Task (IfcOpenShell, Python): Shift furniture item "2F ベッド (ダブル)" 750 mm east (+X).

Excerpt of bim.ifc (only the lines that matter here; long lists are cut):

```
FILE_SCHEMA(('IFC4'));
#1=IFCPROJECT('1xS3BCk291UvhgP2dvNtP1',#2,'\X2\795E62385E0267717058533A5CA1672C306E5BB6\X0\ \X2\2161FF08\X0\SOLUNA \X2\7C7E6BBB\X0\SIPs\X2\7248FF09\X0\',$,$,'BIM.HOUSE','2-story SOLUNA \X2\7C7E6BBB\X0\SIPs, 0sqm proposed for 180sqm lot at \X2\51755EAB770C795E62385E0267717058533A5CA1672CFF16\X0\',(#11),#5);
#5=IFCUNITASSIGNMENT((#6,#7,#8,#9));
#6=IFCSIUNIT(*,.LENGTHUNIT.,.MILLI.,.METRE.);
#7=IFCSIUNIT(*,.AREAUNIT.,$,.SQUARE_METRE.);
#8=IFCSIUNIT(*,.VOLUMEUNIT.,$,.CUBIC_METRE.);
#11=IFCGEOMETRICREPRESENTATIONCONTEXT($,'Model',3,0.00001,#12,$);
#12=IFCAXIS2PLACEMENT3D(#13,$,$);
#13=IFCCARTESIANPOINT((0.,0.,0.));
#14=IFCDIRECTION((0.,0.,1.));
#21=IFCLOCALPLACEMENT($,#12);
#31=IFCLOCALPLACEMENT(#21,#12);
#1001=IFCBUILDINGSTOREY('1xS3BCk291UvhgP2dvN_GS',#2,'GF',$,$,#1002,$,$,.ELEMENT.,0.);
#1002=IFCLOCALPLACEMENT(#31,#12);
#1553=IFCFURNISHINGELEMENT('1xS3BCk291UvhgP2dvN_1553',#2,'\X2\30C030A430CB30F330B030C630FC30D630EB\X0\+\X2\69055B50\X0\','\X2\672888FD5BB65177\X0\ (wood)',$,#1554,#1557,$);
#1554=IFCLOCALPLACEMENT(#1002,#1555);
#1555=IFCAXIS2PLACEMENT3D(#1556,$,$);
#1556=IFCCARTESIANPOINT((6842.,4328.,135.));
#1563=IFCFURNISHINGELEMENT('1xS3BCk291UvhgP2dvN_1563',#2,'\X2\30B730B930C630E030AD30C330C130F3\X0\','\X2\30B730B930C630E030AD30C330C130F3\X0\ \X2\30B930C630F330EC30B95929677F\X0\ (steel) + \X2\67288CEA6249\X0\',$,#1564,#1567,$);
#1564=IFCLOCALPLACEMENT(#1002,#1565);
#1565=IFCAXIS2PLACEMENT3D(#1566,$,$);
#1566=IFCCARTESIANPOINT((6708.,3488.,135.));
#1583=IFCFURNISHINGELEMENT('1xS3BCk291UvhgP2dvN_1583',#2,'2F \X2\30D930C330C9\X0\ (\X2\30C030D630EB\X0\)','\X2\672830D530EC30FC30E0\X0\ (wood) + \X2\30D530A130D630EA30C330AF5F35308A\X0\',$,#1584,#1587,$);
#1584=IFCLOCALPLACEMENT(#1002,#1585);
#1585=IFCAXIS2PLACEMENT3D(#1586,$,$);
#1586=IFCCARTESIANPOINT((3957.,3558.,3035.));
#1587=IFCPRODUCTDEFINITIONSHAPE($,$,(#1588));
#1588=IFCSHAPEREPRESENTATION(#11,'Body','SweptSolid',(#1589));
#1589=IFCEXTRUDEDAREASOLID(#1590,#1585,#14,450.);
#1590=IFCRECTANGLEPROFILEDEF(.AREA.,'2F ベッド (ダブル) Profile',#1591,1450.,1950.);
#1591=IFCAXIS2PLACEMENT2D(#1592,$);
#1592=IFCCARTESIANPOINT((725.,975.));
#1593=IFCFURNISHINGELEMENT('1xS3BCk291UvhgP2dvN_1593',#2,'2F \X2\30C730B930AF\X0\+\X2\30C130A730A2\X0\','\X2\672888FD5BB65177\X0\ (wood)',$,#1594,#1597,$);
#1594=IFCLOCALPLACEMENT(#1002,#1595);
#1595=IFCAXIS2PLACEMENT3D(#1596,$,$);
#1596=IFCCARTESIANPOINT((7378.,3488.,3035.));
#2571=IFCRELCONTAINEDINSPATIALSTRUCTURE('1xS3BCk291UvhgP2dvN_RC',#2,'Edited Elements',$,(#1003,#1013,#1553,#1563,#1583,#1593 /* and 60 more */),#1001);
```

```python
import ifcopenshell
import ifcopenshell.api.geometry
import ifcopenshell.util.placement
import ifcopenshell.util.unit

model = ifcopenshell.open("bim.ifc")
unit_scale = ifcopenshell.util.unit.calculate_unit_scale(model)

item = model.by_id(1583)
matrix = ifcopenshell.util.placement.get_local_placement(item.ObjectPlacement)
matrix[0, 3] += 0.75 / unit_scale
ifcopenshell.api.geometry.edit_object_placement(model, product=item, matrix=matrix, is_si=False)

print(ifcopenshell.util.placement.get_local_placement(item.ObjectPlacement).round(3) + 0.0)

model.write("bim_edited.ifc")
```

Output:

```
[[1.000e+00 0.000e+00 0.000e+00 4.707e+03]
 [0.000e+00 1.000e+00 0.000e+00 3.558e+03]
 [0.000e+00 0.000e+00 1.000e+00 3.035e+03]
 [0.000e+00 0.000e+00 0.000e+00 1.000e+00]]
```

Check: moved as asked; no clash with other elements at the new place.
